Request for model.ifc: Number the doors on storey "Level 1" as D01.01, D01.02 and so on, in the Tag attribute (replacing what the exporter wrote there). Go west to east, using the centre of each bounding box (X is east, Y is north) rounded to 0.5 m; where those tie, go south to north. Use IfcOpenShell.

First a look at what the model holds.

```python
import ifcopenshell
import ifcopenshell.util.element
import ifcopenshell.util.placement

model = ifcopenshell.open("model.ifc")
print(model.schema)
storey = next(s for s in model.by_type("IfcBuildingStorey") if s.Name == "Level 1")
doors = [e for e in ifcopenshell.util.element.get_decomposition(storey) if e.is_a("IfcDoor")]
for e in sorted(doors, key=lambda e: e.id()):
    origin = ifcopenshell.util.placement.get_local_placement(e.ObjectPlacement)[:3, 3]
    print(e.id(), e.Tag, e.Name, origin.round(2) + 0.0, sep=" | ")
```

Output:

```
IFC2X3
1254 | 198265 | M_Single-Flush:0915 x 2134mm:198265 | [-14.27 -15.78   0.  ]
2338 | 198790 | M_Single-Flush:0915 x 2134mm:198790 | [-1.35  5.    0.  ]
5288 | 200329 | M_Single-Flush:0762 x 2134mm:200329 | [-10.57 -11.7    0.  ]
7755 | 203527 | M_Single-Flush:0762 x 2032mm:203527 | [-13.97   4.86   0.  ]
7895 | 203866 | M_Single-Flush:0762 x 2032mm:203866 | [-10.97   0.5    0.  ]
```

```python
import ifcopenshell
import ifcopenshell.geom
import ifcopenshell.util.element
import ifcopenshell.util.shape

model = ifcopenshell.open("model.ifc")
settings = ifcopenshell.geom.settings()
settings.set("use-world-coords", True)


def centre(element):
    shape = ifcopenshell.geom.create_shape(settings, element)
    return ifcopenshell.util.shape.get_bbox_centroid(shape.geometry)


storey = next(s for s in model.by_type("IfcBuildingStorey") if s.Name == "Level 1")
doors = [e for e in ifcopenshell.util.element.get_decomposition(storey) if e.is_a("IfcDoor")]

# Insertion points can sit at a corner or the storey origin, so sort by the geometry (in metres).
centres = {e: centre(e) for e in doors}
doors.sort(key=lambda e: (round(centres[e][0] / 0.5), centres[e][1]))

for i, e in enumerate(doors, start=1):
    number = f"D01.{i:02d}"
    e.Tag = number
    print(e.id(), number)

model.write("model_edited.ifc")
```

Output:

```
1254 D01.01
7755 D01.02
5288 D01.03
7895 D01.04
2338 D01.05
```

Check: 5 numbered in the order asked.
